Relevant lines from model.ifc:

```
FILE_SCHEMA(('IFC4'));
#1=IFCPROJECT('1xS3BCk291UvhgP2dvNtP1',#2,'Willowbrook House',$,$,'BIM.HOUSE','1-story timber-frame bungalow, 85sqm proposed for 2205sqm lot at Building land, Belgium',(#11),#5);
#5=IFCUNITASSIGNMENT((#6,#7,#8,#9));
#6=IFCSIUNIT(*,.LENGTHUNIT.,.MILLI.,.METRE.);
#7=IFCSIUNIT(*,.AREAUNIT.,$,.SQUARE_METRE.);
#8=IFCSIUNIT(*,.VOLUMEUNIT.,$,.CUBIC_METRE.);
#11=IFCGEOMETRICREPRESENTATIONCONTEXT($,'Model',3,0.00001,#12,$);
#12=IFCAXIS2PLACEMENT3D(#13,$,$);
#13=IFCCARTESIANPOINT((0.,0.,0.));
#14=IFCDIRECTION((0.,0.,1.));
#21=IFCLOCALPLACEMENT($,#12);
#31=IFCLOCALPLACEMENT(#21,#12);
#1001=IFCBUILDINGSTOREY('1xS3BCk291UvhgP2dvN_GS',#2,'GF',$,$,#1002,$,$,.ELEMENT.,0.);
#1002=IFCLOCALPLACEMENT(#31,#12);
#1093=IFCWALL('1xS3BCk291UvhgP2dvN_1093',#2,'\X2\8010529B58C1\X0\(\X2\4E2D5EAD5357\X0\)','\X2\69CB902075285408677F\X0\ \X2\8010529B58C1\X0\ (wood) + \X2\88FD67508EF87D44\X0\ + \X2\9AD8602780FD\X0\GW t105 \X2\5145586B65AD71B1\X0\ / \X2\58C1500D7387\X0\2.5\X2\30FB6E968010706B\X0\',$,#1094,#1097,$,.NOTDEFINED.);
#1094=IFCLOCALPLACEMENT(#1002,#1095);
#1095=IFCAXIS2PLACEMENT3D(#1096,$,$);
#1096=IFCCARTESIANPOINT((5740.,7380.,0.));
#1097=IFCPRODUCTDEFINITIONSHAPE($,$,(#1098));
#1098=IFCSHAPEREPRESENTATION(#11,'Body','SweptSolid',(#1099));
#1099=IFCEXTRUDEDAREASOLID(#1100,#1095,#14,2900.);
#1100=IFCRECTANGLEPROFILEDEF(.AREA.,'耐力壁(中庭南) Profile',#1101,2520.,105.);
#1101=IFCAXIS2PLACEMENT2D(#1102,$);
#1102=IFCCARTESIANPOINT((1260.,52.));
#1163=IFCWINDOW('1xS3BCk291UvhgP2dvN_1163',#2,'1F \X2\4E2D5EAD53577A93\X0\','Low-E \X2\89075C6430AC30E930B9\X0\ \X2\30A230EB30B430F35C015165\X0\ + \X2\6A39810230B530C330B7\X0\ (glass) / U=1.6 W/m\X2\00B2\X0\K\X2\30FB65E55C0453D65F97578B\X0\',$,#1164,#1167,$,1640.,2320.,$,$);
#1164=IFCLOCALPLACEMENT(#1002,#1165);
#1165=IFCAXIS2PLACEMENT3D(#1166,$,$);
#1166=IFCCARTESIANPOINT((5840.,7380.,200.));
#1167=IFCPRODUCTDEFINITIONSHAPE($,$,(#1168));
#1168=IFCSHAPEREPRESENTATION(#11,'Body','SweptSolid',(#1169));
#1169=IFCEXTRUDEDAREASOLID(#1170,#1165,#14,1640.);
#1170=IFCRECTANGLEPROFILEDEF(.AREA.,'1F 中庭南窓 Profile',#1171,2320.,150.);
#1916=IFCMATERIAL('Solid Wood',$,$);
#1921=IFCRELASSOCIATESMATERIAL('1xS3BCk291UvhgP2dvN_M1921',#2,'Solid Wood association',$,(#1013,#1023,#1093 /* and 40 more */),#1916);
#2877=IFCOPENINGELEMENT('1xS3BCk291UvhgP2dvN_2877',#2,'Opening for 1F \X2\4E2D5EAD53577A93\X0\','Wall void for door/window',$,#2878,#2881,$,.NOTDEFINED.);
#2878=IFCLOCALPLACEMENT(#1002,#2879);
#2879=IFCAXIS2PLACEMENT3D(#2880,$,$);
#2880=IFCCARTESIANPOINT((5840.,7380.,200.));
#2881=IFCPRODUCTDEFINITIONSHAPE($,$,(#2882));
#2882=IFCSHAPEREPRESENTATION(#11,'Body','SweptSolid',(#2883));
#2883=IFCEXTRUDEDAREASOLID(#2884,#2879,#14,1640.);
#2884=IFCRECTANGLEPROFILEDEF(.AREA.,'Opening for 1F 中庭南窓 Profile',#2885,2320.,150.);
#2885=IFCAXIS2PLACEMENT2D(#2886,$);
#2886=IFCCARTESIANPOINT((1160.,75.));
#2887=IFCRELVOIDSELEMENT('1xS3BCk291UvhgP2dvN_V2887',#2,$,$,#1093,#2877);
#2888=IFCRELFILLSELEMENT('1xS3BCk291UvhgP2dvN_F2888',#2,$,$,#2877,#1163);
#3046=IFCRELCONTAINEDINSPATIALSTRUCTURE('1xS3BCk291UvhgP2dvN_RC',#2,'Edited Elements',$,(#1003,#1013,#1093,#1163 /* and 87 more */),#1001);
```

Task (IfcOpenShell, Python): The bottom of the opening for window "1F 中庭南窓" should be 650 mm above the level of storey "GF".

```python
import numpy as np
import ifcopenshell
import ifcopenshell.api.geometry
import ifcopenshell.geom
import ifcopenshell.util.element
import ifcopenshell.util.placement
import ifcopenshell.util.shape
import ifcopenshell.util.unit

model = ifcopenshell.open("model.ifc")
unit_scale = ifcopenshell.util.unit.calculate_unit_scale(model)

window = model.by_guid("1xS3BCk291UvhgP2dvN_1163")
opening = window.FillsVoids[0].RelatingOpeningElement
storey = ifcopenshell.util.element.get_container(window, ifc_class="IfcBuildingStorey")
level = ifcopenshell.util.placement.get_local_placement(storey.ObjectPlacement)[2, 3]

# The opening's origin need not be at the sill, so measure its lowest point.
shape = ifcopenshell.geom.create_shape(ifcopenshell.geom.settings(), opening)
bottom = ifcopenshell.util.shape.get_shape_bottom_elevation(shape, shape.geometry) / unit_scale
dz = level + 650.0 - bottom

shift = np.array([0.0, 0.0, dz])
# The window is not placed relative to its opening, so move both.
for product in (opening, window):
    matrix = ifcopenshell.util.placement.get_local_placement(product.ObjectPlacement)
    matrix[:3, 3] += shift
    ifcopenshell.api.geometry.edit_object_placement(model, product=product, matrix=matrix, is_si=False)

print(f"moved by {dz * unit_scale:+.3f} m")

model.write("model_rev.ifc")
```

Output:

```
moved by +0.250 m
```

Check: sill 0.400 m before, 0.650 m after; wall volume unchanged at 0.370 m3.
